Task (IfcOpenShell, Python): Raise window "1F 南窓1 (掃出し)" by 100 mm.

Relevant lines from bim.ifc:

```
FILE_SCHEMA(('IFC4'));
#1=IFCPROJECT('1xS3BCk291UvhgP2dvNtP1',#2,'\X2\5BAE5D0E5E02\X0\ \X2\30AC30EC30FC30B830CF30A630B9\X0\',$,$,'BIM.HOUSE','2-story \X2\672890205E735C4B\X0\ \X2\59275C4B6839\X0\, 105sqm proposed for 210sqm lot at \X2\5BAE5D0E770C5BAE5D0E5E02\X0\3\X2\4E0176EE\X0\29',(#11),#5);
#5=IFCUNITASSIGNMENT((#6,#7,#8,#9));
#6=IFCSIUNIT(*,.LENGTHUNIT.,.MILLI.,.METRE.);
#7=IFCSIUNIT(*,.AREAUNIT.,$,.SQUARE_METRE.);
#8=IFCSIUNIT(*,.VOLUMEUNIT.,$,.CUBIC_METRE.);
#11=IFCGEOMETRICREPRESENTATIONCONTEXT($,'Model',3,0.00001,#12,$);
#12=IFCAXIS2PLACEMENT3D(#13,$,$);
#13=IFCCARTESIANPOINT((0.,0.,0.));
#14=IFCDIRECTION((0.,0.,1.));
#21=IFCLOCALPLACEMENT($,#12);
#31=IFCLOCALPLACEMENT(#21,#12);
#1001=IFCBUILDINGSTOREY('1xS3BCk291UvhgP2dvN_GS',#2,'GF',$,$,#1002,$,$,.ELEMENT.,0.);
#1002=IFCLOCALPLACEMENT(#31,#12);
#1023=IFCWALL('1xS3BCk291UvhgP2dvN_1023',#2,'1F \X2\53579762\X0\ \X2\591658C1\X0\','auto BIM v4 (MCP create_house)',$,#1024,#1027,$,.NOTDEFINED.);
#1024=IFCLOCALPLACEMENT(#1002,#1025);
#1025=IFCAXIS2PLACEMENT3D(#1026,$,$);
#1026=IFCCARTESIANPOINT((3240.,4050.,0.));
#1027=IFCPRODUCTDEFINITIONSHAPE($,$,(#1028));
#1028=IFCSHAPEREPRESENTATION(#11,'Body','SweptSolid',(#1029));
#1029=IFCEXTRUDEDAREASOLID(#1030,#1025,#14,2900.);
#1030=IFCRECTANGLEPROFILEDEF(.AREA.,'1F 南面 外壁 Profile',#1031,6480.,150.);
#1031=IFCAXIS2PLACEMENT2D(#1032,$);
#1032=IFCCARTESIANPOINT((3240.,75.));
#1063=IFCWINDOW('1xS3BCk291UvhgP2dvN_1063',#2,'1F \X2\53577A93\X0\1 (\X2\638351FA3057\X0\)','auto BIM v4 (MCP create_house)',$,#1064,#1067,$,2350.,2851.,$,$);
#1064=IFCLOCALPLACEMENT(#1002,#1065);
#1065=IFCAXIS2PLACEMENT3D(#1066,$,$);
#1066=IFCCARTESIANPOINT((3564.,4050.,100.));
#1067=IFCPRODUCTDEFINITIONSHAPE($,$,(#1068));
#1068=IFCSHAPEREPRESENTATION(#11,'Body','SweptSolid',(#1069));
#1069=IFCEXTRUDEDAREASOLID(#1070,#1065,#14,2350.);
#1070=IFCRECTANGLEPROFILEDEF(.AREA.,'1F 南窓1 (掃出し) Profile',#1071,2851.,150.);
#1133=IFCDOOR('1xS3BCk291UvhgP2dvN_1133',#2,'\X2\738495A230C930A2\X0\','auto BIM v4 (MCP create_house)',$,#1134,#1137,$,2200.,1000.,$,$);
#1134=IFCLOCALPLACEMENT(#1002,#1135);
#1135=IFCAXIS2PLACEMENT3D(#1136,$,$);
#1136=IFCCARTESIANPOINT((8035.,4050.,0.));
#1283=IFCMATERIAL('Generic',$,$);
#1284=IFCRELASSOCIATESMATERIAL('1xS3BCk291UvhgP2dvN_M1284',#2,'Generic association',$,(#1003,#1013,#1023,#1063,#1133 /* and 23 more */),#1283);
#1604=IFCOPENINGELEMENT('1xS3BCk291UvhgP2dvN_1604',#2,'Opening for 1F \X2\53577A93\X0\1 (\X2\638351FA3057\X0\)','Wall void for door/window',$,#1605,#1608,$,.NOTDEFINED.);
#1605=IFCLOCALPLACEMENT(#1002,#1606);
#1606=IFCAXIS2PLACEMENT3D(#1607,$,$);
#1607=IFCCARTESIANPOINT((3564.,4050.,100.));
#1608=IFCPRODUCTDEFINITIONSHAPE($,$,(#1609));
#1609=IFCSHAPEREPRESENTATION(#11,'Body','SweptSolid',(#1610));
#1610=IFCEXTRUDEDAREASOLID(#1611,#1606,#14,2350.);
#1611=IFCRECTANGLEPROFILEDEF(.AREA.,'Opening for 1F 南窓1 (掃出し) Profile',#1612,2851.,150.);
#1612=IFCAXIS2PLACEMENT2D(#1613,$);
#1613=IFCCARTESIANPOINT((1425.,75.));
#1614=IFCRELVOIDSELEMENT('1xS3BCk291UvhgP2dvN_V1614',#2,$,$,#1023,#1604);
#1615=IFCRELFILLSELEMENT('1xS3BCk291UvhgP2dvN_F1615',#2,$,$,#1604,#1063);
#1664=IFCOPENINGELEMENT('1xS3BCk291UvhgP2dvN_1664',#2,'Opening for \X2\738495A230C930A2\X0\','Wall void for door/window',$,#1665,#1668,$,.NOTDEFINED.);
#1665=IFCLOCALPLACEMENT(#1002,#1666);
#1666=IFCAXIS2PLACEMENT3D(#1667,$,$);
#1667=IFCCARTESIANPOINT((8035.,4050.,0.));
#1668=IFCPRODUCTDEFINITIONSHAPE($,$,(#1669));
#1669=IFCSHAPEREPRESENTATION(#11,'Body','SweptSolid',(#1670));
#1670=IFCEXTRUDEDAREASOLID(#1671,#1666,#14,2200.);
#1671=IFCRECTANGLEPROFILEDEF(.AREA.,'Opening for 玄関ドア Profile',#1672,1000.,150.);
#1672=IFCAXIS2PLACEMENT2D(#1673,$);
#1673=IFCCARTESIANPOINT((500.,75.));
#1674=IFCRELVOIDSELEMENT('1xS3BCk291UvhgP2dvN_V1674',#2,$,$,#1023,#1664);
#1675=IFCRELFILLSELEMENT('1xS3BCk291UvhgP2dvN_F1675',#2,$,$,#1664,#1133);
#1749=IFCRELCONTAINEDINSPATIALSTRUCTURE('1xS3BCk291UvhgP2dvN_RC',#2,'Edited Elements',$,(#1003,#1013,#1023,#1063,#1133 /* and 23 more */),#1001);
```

```python
import numpy as np
import ifcopenshell
import ifcopenshell.api.geometry
import ifcopenshell.util.placement
import ifcopenshell.util.unit

model = ifcopenshell.open("bim.ifc")
unit_scale = ifcopenshell.util.unit.calculate_unit_scale(model)

window = model.by_guid("1xS3BCk291UvhgP2dvN_1063")
opening = window.FillsVoids[0].RelatingOpeningElement
dz = 0.1 / unit_scale

shift = np.array([0.0, 0.0, dz])
# The window is not placed relative to its opening, so move both.
for product in (opening, window):
    matrix = ifcopenshell.util.placement.get_local_placement(product.ObjectPlacement)
    matrix[:3, 3] += shift
    ifcopenshell.api.geometry.edit_object_placement(model, product=product, matrix=matrix, is_si=False)

print(f"moved by {dz * unit_scale:+.3f} m")

model.write("bim-out.ifc")
```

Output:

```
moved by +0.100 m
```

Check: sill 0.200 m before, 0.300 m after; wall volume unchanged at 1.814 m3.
